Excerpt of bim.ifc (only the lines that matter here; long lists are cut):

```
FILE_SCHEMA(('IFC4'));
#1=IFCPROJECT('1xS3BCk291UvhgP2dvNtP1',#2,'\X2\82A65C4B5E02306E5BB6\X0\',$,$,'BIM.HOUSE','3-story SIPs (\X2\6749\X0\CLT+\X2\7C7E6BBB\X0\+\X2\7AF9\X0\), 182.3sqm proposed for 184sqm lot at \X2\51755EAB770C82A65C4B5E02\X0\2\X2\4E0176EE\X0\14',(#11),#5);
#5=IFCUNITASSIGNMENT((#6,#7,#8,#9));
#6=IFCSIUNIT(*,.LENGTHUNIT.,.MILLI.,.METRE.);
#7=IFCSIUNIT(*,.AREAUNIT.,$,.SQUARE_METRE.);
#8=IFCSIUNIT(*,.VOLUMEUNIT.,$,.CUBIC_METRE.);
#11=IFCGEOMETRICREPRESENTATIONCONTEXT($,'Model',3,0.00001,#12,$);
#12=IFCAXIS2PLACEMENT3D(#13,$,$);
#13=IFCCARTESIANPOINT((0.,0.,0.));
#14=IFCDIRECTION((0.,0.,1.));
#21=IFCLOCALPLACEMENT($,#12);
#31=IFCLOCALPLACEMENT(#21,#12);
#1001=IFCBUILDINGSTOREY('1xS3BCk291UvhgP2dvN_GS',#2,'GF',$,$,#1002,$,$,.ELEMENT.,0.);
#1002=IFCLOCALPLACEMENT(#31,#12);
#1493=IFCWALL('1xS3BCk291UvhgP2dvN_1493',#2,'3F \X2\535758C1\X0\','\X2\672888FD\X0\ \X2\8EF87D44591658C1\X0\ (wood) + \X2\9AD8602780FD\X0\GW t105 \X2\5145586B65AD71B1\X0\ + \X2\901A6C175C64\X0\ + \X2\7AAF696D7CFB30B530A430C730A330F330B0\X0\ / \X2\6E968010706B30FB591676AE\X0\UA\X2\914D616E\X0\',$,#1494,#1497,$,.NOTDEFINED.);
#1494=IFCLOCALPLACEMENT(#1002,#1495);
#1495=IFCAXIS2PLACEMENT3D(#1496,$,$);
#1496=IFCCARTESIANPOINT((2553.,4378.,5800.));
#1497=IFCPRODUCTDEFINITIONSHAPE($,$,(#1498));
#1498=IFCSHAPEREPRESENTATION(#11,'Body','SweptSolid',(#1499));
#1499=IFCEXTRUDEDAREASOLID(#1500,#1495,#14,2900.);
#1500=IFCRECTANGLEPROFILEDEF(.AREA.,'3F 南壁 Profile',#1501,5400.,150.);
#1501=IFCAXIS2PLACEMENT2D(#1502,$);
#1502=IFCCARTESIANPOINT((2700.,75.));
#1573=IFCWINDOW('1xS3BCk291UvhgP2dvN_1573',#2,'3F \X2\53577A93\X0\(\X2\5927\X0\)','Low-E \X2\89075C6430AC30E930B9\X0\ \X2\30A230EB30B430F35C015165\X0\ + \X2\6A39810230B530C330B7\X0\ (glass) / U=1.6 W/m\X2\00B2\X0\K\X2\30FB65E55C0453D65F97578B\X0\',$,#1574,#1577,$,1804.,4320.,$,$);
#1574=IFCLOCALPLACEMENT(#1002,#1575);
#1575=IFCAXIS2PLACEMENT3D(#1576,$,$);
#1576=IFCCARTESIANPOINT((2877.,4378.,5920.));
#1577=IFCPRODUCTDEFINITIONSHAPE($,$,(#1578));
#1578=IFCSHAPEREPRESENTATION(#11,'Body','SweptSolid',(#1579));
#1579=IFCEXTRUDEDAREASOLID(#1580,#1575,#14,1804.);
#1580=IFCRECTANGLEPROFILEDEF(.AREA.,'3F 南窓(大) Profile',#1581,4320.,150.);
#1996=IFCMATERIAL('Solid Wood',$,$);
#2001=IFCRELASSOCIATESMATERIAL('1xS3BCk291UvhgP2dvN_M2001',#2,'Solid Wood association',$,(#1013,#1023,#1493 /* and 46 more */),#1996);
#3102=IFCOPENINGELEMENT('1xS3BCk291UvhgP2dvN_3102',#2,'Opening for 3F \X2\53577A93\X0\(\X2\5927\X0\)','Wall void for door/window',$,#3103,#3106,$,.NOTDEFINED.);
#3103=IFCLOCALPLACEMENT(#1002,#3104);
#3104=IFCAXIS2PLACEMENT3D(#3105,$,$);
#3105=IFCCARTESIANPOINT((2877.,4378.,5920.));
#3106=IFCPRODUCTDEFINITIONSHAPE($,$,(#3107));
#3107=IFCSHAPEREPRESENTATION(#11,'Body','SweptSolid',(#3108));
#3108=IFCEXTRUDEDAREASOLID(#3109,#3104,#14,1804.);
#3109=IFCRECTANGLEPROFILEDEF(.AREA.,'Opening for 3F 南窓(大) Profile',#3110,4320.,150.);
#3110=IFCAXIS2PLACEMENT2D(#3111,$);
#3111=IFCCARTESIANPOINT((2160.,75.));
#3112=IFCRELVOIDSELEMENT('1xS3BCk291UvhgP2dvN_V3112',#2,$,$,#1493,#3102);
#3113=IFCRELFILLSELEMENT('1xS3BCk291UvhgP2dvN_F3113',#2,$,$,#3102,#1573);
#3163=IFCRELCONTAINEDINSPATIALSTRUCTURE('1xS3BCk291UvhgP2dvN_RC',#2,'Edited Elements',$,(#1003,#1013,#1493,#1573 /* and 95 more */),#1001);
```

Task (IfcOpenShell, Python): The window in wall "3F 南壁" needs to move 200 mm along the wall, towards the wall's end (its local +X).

```python
import ifcopenshell
import ifcopenshell.api.geometry
import ifcopenshell.util.placement
import ifcopenshell.util.unit

model = ifcopenshell.open("bim.ifc")
unit_scale = ifcopenshell.util.unit.calculate_unit_scale(model)

window = model.by_guid("1xS3BCk291UvhgP2dvN_1573")
opening = window.FillsVoids[0].RelatingOpeningElement
wall = opening.VoidsElements[0].RelatingBuildingElement

wall_matrix = ifcopenshell.util.placement.get_local_placement(wall.ObjectPlacement)
shift = wall_matrix[:3, 0] * 0.2 / unit_scale
before = ifcopenshell.util.placement.get_local_placement(window.ObjectPlacement)[:3, 3].copy()

# The window is not placed relative to its opening, so move both.
for product in (opening, window):
    matrix = ifcopenshell.util.placement.get_local_placement(product.ObjectPlacement)
    matrix[:3, 3] += shift
    ifcopenshell.api.geometry.edit_object_placement(model, product=product, matrix=matrix, is_si=False)

after = ifcopenshell.util.placement.get_local_placement(window.ObjectPlacement)[:3, 3]
print("window moved by", (after - before).round(3) + 0.0)

model.write("bim_v2.ifc")
```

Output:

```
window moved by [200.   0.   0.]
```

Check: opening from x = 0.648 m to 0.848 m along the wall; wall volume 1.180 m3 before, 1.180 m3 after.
